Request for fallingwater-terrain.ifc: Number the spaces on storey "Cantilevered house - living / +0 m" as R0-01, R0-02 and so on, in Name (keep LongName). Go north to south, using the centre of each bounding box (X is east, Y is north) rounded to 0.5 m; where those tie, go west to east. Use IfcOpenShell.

First a look at what the model holds.

```python
import ifcopenshell
import ifcopenshell.util.element
import ifcopenshell.util.placement

model = ifcopenshell.open("fallingwater-terrain.ifc")
print(model.schema)
storey = next(s for s in model.by_type("IfcBuildingStorey") if s.Name == "Cantilevered house - living / +0 m")
spaces = [e for e in ifcopenshell.util.element.get_decomposition(storey) if e.is_a("IfcSpace")]
for e in sorted(spaces, key=lambda e: e.id()):
    origin = ifcopenshell.util.placement.get_local_placement(e.ObjectPlacement)[:3, 3]
    print(e.id(), e.Name, e.LongName, origin.round(2) + 0.0, sep=" | ")
```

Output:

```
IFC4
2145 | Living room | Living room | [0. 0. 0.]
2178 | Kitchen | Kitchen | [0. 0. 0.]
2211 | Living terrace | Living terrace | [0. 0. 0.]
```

```python
import ifcopenshell
import ifcopenshell.geom
import ifcopenshell.util.element
import ifcopenshell.util.shape

model = ifcopenshell.open("fallingwater-terrain.ifc")
settings = ifcopenshell.geom.settings()
settings.set("use-world-coords", True)


def centre(element):
    shape = ifcopenshell.geom.create_shape(settings, element)
    return ifcopenshell.util.shape.get_bbox_centroid(shape.geometry)


storey = next(s for s in model.by_type("IfcBuildingStorey") if s.Name == "Cantilevered house - living / +0 m")
spaces = [e for e in ifcopenshell.util.element.get_decomposition(storey) if e.is_a("IfcSpace")]

# Insertion points can sit at a corner or the storey origin, so sort by the geometry (in metres).
centres = {e: centre(e) for e in spaces}
spaces.sort(key=lambda e: (-round(centres[e][1] / 0.5), centres[e][0]))

for i, e in enumerate(spaces, start=1):
    number = f"R0-{i:02d}"
    e.Name = number
    print(e.id(), number)

model.write("fallingwater-terrain-out.ifc")
```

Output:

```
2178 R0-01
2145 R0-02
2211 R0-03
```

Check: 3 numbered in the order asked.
